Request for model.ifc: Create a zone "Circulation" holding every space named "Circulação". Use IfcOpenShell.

First a look at what the model holds.

```python
import ifcopenshell

model = ifcopenshell.open("model.ifc")
print(model.schema)
seen = {}
for space in model.by_type("IfcSpace"):
    seen[space.LongName] = seen.get(space.LongName, 0) + 1
for name, count in sorted(seen.items(), key=str):
    print(count, "x", name)
print("zones:", [z.Name for z in model.by_type("IfcZone")][:20])
```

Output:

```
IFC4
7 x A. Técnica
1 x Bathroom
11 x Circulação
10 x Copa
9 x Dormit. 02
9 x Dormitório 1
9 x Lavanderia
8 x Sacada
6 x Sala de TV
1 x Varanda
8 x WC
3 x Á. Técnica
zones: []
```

```python
import ifcopenshell
import ifcopenshell.api.group
import ifcopenshell.api.root

model = ifcopenshell.open("model.ifc")

names = {"Circulação"}
spaces = [s for s in model.by_type("IfcSpace") if s.LongName in names]

zone = ifcopenshell.api.root.create_entity(model, ifc_class="IfcZone", name="Circulation")
ifcopenshell.api.group.assign_group(model, products=spaces, group=zone)
print(len(spaces), "spaces in", zone.Name)

model.write("model_rev.ifc")
```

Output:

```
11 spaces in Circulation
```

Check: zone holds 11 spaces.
